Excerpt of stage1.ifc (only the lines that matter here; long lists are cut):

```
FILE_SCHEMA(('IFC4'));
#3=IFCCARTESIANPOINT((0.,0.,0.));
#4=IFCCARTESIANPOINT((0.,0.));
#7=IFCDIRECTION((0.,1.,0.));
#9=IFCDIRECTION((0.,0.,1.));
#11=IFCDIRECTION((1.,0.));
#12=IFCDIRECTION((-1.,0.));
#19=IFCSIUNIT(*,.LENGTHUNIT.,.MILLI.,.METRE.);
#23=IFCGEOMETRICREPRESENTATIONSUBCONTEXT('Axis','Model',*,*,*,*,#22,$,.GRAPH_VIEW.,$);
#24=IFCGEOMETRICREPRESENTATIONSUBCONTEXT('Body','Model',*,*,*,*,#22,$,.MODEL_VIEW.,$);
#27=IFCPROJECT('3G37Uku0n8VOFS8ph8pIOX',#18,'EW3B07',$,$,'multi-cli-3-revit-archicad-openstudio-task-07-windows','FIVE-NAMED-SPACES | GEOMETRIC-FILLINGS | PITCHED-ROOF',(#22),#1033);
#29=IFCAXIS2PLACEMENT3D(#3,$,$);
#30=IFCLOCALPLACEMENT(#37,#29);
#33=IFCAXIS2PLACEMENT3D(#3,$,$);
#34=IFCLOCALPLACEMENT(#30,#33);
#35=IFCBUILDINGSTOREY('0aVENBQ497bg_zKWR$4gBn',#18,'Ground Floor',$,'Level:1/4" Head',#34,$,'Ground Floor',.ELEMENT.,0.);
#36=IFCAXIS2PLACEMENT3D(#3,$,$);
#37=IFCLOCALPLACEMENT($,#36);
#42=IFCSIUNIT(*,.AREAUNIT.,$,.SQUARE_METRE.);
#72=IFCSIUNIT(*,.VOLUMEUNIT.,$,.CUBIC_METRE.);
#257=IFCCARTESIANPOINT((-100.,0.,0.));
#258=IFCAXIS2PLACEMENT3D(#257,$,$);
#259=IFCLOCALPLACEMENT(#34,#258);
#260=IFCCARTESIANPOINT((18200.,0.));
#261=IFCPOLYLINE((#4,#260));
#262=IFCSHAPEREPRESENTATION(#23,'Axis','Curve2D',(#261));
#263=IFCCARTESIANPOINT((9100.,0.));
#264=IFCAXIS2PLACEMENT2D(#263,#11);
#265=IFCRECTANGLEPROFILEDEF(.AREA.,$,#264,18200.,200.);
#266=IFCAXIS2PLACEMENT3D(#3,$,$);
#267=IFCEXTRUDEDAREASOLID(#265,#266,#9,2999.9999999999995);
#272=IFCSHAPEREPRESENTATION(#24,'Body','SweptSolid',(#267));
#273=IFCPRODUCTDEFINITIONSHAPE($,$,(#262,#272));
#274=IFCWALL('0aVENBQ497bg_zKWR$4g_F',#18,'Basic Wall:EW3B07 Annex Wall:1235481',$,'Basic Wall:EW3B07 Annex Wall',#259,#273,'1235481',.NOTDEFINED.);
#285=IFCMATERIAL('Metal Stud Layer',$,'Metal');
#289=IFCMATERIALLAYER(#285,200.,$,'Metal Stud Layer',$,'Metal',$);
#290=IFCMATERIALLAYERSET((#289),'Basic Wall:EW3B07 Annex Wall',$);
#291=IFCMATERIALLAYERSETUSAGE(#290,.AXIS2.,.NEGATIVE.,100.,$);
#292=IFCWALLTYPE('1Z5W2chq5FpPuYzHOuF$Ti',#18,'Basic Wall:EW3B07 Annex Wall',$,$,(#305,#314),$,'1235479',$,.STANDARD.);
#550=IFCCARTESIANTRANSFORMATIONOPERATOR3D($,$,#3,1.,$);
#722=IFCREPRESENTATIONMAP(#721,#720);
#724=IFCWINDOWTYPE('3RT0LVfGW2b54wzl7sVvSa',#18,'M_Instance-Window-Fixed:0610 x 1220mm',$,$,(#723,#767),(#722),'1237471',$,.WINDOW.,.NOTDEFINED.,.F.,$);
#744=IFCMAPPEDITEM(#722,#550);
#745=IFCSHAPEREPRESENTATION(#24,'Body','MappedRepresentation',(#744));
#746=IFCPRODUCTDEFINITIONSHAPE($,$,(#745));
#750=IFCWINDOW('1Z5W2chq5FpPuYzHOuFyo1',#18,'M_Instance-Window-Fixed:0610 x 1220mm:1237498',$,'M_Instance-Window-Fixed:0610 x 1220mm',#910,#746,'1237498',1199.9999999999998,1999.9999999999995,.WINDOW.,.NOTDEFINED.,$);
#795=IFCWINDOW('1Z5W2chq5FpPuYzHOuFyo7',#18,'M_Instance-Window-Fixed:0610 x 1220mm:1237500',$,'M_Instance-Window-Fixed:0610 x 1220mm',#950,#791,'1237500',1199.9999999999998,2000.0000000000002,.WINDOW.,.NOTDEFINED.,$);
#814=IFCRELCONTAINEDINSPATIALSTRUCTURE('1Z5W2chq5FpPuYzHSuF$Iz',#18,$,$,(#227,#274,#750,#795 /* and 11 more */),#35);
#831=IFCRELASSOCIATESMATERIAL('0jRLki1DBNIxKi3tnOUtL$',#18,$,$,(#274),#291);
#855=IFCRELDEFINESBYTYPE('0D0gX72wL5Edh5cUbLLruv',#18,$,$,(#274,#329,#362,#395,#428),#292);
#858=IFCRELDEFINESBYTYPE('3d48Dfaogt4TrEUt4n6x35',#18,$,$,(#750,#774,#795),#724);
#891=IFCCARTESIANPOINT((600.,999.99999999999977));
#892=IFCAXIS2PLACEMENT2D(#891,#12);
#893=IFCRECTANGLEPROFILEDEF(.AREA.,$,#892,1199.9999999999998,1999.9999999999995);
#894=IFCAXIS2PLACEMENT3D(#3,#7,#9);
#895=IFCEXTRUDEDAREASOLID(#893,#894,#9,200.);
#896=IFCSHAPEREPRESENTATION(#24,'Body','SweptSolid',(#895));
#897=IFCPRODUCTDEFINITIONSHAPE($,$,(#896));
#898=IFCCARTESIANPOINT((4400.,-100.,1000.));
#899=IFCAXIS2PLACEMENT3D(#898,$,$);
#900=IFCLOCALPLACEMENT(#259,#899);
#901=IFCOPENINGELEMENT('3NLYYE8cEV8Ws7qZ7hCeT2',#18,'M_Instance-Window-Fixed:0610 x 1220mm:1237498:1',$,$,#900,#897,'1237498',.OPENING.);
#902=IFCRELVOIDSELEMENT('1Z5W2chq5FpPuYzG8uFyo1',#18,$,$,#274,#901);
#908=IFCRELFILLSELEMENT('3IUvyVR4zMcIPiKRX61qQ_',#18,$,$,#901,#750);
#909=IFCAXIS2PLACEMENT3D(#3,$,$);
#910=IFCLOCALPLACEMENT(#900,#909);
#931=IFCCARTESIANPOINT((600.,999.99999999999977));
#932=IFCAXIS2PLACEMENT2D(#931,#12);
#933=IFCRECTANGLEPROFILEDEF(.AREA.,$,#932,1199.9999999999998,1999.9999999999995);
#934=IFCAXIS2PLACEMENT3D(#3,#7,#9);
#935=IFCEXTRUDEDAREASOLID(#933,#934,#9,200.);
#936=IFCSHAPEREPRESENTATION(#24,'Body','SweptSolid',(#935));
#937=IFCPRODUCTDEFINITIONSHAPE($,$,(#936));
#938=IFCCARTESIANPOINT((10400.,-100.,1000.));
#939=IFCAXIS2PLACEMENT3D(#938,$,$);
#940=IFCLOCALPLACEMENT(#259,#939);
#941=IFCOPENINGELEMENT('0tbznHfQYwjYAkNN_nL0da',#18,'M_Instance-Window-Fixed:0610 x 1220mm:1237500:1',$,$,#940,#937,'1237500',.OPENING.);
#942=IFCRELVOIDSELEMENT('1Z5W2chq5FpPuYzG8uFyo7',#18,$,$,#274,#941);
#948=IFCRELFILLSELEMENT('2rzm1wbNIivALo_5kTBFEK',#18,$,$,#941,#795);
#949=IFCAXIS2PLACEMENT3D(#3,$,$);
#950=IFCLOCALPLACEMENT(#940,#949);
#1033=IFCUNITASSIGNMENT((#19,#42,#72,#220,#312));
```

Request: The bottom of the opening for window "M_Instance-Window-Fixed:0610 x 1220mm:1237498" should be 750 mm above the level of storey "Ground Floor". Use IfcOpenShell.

```python
import numpy as np
import ifcopenshell
import ifcopenshell.api.geometry
import ifcopenshell.geom
import ifcopenshell.util.element
import ifcopenshell.util.placement
import ifcopenshell.util.shape
import ifcopenshell.util.unit

model = ifcopenshell.open("stage1.ifc")
unit_scale = ifcopenshell.util.unit.calculate_unit_scale(model)

window = model.by_id(750)
opening = window.FillsVoids[0].RelatingOpeningElement
storey = ifcopenshell.util.element.get_container(window, ifc_class="IfcBuildingStorey")
level = ifcopenshell.util.placement.get_local_placement(storey.ObjectPlacement)[2, 3]

# The opening's origin need not be at the sill, so measure its lowest point.
shape = ifcopenshell.geom.create_shape(ifcopenshell.geom.settings(), opening)
bottom = ifcopenshell.util.shape.get_shape_bottom_elevation(shape, shape.geometry) / unit_scale
dz = level + 0.75 / unit_scale - bottom

shift = np.array([0.0, 0.0, dz])
# The window is placed relative to its opening, so it follows when the opening moves.
matrix = ifcopenshell.util.placement.get_local_placement(opening.ObjectPlacement)
matrix[:3, 3] += shift
ifcopenshell.api.geometry.edit_object_placement(
    model, product=opening, matrix=matrix, is_si=False, should_transform_children=True
)

print(f"moved by {dz * unit_scale:+.3f} m")

model.write("stage1_v2.ifc")
```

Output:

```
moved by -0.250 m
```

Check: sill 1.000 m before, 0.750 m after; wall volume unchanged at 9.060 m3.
